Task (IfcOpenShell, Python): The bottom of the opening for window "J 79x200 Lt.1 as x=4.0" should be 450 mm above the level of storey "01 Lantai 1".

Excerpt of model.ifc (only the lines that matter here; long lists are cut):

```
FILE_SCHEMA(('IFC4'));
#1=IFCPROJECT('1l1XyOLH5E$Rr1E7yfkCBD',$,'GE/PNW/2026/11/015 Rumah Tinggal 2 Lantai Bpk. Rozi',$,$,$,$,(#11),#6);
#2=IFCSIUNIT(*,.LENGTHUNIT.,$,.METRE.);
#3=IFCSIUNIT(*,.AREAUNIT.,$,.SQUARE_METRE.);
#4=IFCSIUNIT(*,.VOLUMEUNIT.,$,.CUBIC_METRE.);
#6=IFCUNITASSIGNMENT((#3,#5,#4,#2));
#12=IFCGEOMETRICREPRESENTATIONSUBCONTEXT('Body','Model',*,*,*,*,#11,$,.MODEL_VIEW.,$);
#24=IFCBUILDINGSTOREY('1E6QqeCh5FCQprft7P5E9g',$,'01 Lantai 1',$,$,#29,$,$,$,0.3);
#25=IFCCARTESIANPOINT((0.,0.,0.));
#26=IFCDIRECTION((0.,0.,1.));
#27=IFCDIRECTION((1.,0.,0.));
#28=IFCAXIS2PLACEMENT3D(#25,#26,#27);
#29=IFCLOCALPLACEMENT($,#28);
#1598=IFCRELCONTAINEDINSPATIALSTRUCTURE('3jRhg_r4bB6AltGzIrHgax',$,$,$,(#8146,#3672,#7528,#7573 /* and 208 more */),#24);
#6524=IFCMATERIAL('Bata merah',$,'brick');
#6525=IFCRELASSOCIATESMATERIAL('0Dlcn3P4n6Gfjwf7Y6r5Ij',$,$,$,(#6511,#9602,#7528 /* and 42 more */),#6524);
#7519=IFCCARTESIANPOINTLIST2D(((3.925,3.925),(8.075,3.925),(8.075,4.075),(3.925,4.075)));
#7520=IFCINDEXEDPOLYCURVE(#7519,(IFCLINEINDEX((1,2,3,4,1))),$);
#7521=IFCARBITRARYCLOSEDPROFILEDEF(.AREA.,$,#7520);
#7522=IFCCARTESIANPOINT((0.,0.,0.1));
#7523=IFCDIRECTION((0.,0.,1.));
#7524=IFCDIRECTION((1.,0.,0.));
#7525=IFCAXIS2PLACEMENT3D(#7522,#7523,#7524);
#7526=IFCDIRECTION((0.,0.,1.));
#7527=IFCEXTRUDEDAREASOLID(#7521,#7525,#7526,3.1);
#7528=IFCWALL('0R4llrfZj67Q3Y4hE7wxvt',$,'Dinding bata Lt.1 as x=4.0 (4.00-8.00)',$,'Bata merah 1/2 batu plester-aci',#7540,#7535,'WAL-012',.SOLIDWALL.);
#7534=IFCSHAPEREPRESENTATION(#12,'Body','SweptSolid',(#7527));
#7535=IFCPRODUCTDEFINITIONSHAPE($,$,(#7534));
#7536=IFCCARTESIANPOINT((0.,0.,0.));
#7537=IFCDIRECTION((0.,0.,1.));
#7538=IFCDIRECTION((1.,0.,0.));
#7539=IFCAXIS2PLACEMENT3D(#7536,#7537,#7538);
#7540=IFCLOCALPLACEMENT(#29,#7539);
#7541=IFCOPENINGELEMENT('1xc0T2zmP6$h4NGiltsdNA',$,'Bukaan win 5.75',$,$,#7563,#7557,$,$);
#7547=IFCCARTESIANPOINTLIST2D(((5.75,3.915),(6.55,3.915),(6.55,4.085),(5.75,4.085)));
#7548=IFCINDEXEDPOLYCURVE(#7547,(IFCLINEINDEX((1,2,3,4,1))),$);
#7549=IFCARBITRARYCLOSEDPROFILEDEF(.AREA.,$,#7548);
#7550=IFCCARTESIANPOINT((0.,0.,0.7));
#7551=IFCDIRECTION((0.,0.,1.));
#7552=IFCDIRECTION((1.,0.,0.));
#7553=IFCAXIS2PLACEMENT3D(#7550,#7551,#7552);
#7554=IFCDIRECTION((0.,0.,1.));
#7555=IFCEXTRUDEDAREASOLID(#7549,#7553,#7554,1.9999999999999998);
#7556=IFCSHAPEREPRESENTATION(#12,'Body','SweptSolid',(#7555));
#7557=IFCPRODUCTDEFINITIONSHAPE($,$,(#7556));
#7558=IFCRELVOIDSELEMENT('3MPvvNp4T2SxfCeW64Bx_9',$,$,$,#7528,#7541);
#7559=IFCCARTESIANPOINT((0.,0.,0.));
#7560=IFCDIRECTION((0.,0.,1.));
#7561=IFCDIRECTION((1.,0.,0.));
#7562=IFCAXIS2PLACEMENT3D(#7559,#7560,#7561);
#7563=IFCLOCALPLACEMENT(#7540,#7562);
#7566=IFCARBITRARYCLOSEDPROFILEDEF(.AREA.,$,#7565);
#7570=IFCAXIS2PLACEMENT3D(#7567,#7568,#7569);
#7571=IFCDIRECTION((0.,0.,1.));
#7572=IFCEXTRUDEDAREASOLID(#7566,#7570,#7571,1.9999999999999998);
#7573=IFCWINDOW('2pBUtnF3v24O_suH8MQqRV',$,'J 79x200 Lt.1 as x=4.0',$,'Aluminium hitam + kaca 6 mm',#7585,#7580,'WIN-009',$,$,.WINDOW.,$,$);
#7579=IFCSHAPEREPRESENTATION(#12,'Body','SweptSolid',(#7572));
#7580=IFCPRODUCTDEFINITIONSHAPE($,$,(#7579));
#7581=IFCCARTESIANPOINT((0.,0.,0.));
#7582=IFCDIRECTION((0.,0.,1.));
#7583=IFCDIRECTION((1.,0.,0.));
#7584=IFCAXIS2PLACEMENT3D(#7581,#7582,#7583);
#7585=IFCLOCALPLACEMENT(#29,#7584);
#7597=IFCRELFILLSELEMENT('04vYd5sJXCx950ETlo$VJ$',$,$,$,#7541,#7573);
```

```python
import numpy as np
import ifcopenshell
import ifcopenshell.api.geometry
import ifcopenshell.geom
import ifcopenshell.util.element
import ifcopenshell.util.placement
import ifcopenshell.util.shape
import ifcopenshell.util.unit

model = ifcopenshell.open("model.ifc")
unit_scale = ifcopenshell.util.unit.calculate_unit_scale(model)

window = model.by_guid("2pBUtnF3v24O_suH8MQqRV")
opening = window.FillsVoids[0].RelatingOpeningElement
storey = ifcopenshell.util.element.get_container(window, ifc_class="IfcBuildingStorey")
level = ifcopenshell.util.placement.get_local_placement(storey.ObjectPlacement)[2, 3]

# The opening's origin need not be at the sill, so measure its lowest point.
shape = ifcopenshell.geom.create_shape(ifcopenshell.geom.settings(), opening)
bottom = ifcopenshell.util.shape.get_shape_bottom_elevation(shape, shape.geometry) / unit_scale
dz = level + 0.45 - bottom

shift = np.array([0.0, 0.0, dz])
# The window is not placed relative to its opening, so move both.
for product in (opening, window):
    matrix = ifcopenshell.util.placement.get_local_placement(product.ObjectPlacement)
    matrix[:3, 3] += shift
    ifcopenshell.api.geometry.edit_object_placement(model, product=product, matrix=matrix, is_si=False)

print(f"moved by {dz * unit_scale:+.3f} m")

model.write("model_updated.ifc")
```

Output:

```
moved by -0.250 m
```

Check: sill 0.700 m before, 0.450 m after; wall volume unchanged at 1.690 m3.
